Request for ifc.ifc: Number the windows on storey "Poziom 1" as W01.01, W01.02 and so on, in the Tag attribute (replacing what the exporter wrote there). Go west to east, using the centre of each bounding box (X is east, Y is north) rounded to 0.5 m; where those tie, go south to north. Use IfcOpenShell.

First a look at what the model holds.

```python
import ifcopenshell
import ifcopenshell.util.element
import ifcopenshell.util.placement

model = ifcopenshell.open("ifc.ifc")
print(model.schema)
storey = next(s for s in model.by_type("IfcBuildingStorey") if s.Name == "Poziom 1")
windows = [e for e in ifcopenshell.util.element.get_decomposition(storey) if e.is_a("IfcWindow")]
for e in sorted(windows, key=lambda e: e.id()):
    origin = ifcopenshell.util.placement.get_local_placement(e.ObjectPlacement)[:3, 3]
    print(e.id(), e.Tag, e.Name, origin.round(2) + 0.0, sep=" | ")
```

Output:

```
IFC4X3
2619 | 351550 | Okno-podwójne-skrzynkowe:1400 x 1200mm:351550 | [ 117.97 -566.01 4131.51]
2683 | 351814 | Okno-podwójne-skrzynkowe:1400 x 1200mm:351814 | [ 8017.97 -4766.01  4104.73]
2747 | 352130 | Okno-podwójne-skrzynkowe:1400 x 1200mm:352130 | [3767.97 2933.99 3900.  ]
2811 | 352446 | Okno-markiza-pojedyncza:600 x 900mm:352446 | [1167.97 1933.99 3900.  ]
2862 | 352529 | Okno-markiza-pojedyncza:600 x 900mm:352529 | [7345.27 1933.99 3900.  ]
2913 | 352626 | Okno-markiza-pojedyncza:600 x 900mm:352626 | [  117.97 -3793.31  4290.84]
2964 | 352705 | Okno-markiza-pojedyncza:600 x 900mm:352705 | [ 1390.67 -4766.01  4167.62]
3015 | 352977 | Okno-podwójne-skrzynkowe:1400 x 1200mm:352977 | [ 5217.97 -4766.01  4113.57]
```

```python
import ifcopenshell
import ifcopenshell.geom
import ifcopenshell.util.element
import ifcopenshell.util.shape

model = ifcopenshell.open("ifc.ifc")
settings = ifcopenshell.geom.settings()
settings.set("use-world-coords", True)


def centre(element):
    shape = ifcopenshell.geom.create_shape(settings, element)
    return ifcopenshell.util.shape.get_bbox_centroid(shape.geometry)


storey = next(s for s in model.by_type("IfcBuildingStorey") if s.Name == "Poziom 1")
windows = [e for e in ifcopenshell.util.element.get_decomposition(storey) if e.is_a("IfcWindow")]

# Insertion points can sit at a corner or the storey origin, so sort by the geometry (in metres).
centres = {e: centre(e) for e in windows}
windows.sort(key=lambda e: (round(centres[e][0] / 0.5), centres[e][1]))

for i, e in enumerate(windows, start=1):
    number = f"W01.{i:02d}"
    e.Tag = number
    print(e.id(), number)

model.write("ifc_edited.ifc")
```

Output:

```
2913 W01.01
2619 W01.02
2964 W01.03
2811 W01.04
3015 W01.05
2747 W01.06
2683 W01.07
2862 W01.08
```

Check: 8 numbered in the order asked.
